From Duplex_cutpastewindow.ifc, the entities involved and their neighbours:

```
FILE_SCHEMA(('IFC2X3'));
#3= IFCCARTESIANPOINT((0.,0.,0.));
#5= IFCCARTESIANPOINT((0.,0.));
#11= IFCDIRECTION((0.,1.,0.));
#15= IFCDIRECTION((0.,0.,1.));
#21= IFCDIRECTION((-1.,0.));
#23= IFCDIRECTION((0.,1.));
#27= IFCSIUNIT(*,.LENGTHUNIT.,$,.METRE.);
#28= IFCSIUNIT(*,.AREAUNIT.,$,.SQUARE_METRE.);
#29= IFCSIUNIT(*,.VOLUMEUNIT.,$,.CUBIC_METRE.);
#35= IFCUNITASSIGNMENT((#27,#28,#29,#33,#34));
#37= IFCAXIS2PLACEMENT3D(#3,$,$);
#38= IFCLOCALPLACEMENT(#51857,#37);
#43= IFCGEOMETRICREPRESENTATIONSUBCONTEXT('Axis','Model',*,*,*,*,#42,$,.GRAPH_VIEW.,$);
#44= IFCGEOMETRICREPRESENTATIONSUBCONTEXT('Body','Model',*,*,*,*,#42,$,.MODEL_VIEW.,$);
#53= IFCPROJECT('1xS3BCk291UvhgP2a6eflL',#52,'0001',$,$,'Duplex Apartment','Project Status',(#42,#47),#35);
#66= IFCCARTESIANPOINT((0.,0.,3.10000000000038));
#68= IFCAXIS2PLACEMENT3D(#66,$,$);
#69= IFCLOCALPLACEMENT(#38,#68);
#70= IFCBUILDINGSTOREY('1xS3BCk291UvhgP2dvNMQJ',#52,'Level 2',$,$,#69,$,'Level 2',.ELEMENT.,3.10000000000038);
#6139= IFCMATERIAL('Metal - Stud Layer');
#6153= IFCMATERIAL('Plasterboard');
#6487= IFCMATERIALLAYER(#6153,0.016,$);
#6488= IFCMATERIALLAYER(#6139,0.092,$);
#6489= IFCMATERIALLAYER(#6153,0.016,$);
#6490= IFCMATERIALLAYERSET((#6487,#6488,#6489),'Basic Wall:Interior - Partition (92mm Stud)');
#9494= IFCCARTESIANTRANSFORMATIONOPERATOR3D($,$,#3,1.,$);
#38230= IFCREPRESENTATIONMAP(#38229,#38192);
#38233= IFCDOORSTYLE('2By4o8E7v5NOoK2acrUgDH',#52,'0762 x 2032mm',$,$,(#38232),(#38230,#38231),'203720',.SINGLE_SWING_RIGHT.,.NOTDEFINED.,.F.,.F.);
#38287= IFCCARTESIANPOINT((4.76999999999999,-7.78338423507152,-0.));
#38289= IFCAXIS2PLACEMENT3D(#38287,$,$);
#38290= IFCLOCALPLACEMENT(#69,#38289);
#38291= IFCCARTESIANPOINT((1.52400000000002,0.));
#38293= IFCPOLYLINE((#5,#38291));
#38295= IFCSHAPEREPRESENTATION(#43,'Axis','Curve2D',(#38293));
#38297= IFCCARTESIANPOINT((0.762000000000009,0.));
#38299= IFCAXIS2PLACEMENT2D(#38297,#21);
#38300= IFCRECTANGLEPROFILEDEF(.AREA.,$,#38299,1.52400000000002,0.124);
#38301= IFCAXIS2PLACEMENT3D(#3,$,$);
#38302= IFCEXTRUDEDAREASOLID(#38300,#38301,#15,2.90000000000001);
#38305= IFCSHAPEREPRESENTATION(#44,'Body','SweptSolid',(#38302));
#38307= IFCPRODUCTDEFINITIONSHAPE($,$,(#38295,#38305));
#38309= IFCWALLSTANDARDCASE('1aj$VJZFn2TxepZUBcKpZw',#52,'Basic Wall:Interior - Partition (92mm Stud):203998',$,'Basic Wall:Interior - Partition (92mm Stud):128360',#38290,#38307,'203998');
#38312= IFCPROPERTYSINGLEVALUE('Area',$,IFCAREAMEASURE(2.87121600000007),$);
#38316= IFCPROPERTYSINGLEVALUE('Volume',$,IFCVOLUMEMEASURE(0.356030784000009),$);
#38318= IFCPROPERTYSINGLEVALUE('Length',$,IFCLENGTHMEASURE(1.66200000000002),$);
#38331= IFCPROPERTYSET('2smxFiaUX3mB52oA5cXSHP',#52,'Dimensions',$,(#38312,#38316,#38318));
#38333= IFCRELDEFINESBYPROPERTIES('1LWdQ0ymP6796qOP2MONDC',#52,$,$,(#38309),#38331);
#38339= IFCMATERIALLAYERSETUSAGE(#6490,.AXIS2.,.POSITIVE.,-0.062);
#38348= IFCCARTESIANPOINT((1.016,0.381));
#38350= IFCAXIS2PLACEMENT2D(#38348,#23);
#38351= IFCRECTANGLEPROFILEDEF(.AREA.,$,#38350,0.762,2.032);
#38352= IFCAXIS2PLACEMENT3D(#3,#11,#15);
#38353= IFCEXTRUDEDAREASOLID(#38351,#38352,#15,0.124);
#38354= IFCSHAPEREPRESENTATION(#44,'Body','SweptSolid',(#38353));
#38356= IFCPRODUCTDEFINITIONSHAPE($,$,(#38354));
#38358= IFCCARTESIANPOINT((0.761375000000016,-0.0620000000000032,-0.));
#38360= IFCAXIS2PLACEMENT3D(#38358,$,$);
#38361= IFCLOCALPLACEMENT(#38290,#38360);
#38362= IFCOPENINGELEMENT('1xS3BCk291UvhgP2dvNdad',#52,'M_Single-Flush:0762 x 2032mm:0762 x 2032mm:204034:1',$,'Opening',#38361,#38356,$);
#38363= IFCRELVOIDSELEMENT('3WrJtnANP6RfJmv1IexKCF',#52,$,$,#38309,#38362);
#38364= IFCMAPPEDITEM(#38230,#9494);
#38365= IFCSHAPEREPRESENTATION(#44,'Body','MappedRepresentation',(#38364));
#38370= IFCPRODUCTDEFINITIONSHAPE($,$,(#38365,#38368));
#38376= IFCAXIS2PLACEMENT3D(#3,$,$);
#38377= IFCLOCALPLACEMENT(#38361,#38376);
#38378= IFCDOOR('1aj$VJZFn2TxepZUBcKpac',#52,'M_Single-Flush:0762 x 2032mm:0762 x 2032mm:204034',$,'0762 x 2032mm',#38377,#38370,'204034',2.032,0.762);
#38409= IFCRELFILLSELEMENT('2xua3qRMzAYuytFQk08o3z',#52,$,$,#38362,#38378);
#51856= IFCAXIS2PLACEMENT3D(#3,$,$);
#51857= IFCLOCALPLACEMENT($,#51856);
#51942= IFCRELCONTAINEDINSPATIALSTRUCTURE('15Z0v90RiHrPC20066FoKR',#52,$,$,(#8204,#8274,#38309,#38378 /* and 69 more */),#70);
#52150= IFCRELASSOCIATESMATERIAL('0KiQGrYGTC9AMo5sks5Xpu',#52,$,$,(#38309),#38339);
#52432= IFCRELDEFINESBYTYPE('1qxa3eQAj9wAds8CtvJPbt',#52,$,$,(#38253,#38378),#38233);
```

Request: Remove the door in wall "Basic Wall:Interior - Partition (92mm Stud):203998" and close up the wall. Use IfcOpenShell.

```python
import ifcopenshell
import ifcopenshell.api.feature
import ifcopenshell.api.pset
import ifcopenshell.api.root
import ifcopenshell.geom
import ifcopenshell.util.element
import ifcopenshell.util.shape
import ifcopenshell.util.unit

model = ifcopenshell.open("Duplex_cutpastewindow.ifc")
area_scale = ifcopenshell.util.unit.calculate_unit_scale(model, "AREAUNIT")
volume_scale = ifcopenshell.util.unit.calculate_unit_scale(model, "VOLUMEUNIT")
settings = ifcopenshell.geom.settings()


def volume(element):
    """Net volume in cubic metres, openings subtracted."""
    shape = ifcopenshell.geom.create_shape(settings, element)
    return ifcopenshell.util.shape.get_volume(shape.geometry)


door = model.by_guid("1aj$VJZFn2TxepZUBcKpac")
opening = door.FillsVoids[0].RelatingOpeningElement
wall = opening.VoidsElements[0].RelatingBuildingElement
before = volume(wall)

ifcopenshell.api.root.remove_product(model, product=door)
ifcopenshell.api.feature.remove_feature(model, feature=opening)

after = volume(wall)
thickness = 0.124  # wall thickness in metres

# Update the wall's stored quantities.
pset = model.by_id(ifcopenshell.util.element.get_pset(wall, "Dimensions", should_inherit=False)["id"])
ifcopenshell.api.pset.edit_pset(model, pset=pset, properties={
    "Area": model.create_entity("IfcAreaMeasure", after / thickness / area_scale),
    "Volume": model.create_entity("IfcVolumeMeasure", after / volume_scale),
})

print(f"wall volume {before:.3f} -> {after:.3f} m3")

model.write("Duplex_cutpastewindow_rev.ifc")
```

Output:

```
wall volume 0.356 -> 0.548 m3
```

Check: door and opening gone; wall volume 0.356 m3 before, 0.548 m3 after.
